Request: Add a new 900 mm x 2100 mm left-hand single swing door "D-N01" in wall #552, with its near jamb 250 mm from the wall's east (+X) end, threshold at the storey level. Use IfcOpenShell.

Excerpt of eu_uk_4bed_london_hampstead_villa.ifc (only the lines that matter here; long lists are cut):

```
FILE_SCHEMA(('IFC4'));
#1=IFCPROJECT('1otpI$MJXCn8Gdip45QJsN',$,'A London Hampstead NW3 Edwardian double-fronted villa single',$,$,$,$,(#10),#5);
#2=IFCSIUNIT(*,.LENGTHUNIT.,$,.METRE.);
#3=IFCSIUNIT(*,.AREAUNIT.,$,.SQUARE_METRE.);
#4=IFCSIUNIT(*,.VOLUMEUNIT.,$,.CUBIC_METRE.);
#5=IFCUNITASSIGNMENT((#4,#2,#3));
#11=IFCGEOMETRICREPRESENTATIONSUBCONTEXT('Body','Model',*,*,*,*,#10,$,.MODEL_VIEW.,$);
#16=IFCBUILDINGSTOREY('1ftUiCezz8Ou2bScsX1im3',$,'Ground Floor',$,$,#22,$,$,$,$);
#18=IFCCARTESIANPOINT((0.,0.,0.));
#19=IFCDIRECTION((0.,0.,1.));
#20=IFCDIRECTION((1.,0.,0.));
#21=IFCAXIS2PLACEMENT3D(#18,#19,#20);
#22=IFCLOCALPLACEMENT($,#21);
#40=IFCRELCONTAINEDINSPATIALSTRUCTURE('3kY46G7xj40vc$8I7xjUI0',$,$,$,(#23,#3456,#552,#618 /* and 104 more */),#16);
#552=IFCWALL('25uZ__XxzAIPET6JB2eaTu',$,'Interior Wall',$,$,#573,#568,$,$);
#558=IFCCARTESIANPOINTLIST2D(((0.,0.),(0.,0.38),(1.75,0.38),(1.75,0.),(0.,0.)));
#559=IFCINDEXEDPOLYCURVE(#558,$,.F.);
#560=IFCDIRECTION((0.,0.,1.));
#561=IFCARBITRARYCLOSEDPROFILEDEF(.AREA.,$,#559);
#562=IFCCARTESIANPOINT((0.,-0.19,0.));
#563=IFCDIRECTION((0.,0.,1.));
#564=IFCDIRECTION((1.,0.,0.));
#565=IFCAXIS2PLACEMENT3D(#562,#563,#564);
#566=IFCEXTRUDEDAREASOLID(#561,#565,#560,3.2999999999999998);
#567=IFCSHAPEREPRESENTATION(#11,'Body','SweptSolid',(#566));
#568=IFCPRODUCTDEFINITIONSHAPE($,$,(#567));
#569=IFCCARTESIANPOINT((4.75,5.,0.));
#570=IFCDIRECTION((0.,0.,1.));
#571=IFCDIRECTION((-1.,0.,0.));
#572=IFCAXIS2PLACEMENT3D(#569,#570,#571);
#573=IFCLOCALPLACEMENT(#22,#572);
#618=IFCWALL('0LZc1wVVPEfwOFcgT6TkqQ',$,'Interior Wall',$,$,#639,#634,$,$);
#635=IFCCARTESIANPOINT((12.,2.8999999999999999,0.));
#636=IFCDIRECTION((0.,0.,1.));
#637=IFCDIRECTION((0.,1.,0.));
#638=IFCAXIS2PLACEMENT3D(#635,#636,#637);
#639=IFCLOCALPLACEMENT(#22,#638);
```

```python
import numpy as np
import ifcopenshell
import ifcopenshell.api.feature
import ifcopenshell.api.geometry
import ifcopenshell.api.root
import ifcopenshell.api.spatial
import ifcopenshell.geom
import ifcopenshell.util.element
import ifcopenshell.util.placement
import ifcopenshell.util.representation
import ifcopenshell.util.shape
import ifcopenshell.util.unit

model = ifcopenshell.open("eu_uk_4bed_london_hampstead_villa.ifc")
unit_scale = ifcopenshell.util.unit.calculate_unit_scale(model)
settings = ifcopenshell.geom.settings()


def volume(element):
    """Net volume in cubic metres, openings subtracted."""
    shape = ifcopenshell.geom.create_shape(settings, element)
    return ifcopenshell.util.shape.get_volume(shape.geometry)


wall = model.by_guid("25uZ__XxzAIPET6JB2eaTu")
storey = ifcopenshell.util.element.get_container(wall, ifc_class="IfcBuildingStorey")
context = ifcopenshell.util.representation.get_context(model, "Model", "Body", "MODEL_VIEW")
before = volume(wall)

width, height, from_end, sill = 0.9, 2.1, 0.25, 0.0  # metres

# The wall runs along its own X axis, and the end named is its -X end.
wall_shape = ifcopenshell.geom.create_shape(settings, wall)
x, y, z = ifcopenshell.util.shape.get_vertices(wall_shape.geometry).T
start = x.min() + from_end
face, thickness = float(y.min()), float(y.max() - y.min())
wall_matrix = ifcopenshell.util.placement.get_local_placement(wall.ObjectPlacement)
level = ifcopenshell.util.placement.get_local_placement(storey.ObjectPlacement)[2, 3]


def in_wall(x, y):
    """Placement at x, y metres in the wall's axes, at sill height."""
    matrix = wall_matrix.copy()
    matrix[:, 3] = wall_matrix @ np.array([x / unit_scale, y / unit_scale, 0.0, 1.0])
    matrix[2, 3] = level + sill / unit_scale
    return matrix


# Opening: a box that overshoots both wall faces by 50 mm.
opening = ifcopenshell.api.root.create_entity(model, ifc_class="IfcOpeningElement", predefined_type="OPENING")
box = ifcopenshell.api.geometry.add_wall_representation(
    model, context=context, length=width, height=height, thickness=thickness + 0.1
)
ifcopenshell.api.geometry.assign_representation(model, product=opening, representation=box)
ifcopenshell.api.geometry.edit_object_placement(model, product=opening, matrix=in_wall(start, face - 0.05), is_si=False)
ifcopenshell.api.feature.add_feature(model, feature=opening, element=wall)

door = ifcopenshell.api.root.create_entity(model, ifc_class="IfcDoor", name="D-N01", predefined_type="DOOR")
door.OverallWidth, door.OverallHeight = width / unit_scale, height / unit_scale
door.OperationType = "SINGLE_SWING_LEFT"
body = ifcopenshell.api.geometry.add_door_representation(
    model,
    context=context,
    overall_width=door.OverallWidth,
    overall_height=door.OverallHeight,
    operation_type="SINGLE_SWING_LEFT",
    lining_properties={"LiningDepth": thickness / unit_scale, "ThresholdDepth": thickness / unit_scale},
)
ifcopenshell.api.geometry.assign_representation(model, product=door, representation=body)
ifcopenshell.api.spatial.assign_container(model, products=[door], relating_structure=storey)
ifcopenshell.api.feature.add_filling(model, opening=opening, element=door)

# The lining spans the wall, so the door starts at the wall face.
ifcopenshell.api.geometry.edit_object_placement(model, product=door, matrix=in_wall(start, face), is_si=False)

after = volume(wall)

print(f"wall volume {before:.3f} -> {after:.3f} m3")

model.write("eu_uk_4bed_london_hampstead_villa_edited.ifc")
```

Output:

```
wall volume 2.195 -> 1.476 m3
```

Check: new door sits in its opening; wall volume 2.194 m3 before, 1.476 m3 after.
